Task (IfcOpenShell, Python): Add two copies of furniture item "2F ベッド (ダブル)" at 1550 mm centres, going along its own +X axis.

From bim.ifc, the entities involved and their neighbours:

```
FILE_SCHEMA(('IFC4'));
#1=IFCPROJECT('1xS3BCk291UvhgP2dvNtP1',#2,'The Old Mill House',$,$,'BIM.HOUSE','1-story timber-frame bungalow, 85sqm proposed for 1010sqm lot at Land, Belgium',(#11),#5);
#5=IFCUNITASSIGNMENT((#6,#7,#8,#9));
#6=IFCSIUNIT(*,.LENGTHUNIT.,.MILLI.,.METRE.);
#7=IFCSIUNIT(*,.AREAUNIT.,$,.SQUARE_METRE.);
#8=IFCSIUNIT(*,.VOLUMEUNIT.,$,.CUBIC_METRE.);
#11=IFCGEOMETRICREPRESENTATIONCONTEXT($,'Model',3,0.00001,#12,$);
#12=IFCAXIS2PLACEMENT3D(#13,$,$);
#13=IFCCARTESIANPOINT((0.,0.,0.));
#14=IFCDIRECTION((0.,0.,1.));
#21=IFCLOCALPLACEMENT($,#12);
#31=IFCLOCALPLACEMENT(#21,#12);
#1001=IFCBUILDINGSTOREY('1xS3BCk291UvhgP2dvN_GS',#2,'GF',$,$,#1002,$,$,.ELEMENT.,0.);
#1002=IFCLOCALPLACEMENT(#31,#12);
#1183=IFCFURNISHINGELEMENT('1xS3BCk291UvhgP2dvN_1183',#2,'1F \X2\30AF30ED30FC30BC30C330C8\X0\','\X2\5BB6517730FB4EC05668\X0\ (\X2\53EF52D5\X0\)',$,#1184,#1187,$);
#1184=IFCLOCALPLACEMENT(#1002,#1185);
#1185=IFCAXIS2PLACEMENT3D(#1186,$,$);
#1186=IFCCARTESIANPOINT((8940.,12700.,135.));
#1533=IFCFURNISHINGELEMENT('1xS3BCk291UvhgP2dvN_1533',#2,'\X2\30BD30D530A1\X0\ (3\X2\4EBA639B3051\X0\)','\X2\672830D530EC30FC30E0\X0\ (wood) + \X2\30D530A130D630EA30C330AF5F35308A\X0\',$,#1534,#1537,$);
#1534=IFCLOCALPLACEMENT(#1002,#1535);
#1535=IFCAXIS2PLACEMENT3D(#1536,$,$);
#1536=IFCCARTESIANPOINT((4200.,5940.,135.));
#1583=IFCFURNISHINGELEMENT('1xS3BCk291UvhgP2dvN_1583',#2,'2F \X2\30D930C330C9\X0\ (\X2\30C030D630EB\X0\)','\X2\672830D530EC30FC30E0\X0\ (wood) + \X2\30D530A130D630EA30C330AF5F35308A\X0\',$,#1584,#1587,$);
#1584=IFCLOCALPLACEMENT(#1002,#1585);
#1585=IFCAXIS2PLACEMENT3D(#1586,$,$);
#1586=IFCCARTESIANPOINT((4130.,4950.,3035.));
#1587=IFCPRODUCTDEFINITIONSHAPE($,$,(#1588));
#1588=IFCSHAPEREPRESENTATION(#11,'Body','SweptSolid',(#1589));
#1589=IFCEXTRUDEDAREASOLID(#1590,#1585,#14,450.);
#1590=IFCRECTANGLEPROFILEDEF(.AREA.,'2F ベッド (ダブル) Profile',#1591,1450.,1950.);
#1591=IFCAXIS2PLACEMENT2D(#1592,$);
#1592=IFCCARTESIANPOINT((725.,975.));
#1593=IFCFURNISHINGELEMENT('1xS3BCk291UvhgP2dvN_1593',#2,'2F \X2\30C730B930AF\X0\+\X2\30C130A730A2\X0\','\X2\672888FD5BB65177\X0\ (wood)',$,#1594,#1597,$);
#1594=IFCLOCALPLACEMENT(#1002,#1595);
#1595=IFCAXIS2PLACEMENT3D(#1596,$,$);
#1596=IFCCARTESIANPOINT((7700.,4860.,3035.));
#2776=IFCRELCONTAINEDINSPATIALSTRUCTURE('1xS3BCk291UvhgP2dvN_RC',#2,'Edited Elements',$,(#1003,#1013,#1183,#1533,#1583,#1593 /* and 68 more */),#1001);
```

```python
import ifcopenshell
import ifcopenshell.api.geometry
import ifcopenshell.api.root
import ifcopenshell.util.element
import ifcopenshell.util.placement

model = ifcopenshell.open("bim.ifc")


def reuse_history(source, copy):
    """copy_class also copies each property set's owner history, people and application; keep the originals."""
    for rel in copy.IsDefinedBy:
        if rel.is_a("IfcRelDefinesByProperties") and (history := rel.RelatingPropertyDefinition.OwnerHistory):
            rel.RelatingPropertyDefinition.OwnerHistory = source.OwnerHistory
            ifcopenshell.util.element.remove_deep2(model, history)


source = model.by_guid("1xS3BCk291UvhgP2dvN_1583")
base = ifcopenshell.util.placement.get_local_placement(source.ObjectPlacement)
step = base[:3, 0] * 1550.0

for i in range(1, 3):
    copy = ifcopenshell.api.root.copy_class(model, product=source)
    copy.Representation = ifcopenshell.util.element.copy_deep(
        model, source.Representation, exclude=["IfcGeometricRepresentationContext", "IfcRepresentationMap"]
    )
    reuse_history(source, copy)
    matrix = base.copy()
    matrix[:3, 3] += i * step
    print("added at", matrix[:3, 3].round(3) + 0.0)
    ifcopenshell.api.geometry.edit_object_placement(model, product=copy, matrix=matrix, is_si=False)

model.write("bim-out.ifc")
```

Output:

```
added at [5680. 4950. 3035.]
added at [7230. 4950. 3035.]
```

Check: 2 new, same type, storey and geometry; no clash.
